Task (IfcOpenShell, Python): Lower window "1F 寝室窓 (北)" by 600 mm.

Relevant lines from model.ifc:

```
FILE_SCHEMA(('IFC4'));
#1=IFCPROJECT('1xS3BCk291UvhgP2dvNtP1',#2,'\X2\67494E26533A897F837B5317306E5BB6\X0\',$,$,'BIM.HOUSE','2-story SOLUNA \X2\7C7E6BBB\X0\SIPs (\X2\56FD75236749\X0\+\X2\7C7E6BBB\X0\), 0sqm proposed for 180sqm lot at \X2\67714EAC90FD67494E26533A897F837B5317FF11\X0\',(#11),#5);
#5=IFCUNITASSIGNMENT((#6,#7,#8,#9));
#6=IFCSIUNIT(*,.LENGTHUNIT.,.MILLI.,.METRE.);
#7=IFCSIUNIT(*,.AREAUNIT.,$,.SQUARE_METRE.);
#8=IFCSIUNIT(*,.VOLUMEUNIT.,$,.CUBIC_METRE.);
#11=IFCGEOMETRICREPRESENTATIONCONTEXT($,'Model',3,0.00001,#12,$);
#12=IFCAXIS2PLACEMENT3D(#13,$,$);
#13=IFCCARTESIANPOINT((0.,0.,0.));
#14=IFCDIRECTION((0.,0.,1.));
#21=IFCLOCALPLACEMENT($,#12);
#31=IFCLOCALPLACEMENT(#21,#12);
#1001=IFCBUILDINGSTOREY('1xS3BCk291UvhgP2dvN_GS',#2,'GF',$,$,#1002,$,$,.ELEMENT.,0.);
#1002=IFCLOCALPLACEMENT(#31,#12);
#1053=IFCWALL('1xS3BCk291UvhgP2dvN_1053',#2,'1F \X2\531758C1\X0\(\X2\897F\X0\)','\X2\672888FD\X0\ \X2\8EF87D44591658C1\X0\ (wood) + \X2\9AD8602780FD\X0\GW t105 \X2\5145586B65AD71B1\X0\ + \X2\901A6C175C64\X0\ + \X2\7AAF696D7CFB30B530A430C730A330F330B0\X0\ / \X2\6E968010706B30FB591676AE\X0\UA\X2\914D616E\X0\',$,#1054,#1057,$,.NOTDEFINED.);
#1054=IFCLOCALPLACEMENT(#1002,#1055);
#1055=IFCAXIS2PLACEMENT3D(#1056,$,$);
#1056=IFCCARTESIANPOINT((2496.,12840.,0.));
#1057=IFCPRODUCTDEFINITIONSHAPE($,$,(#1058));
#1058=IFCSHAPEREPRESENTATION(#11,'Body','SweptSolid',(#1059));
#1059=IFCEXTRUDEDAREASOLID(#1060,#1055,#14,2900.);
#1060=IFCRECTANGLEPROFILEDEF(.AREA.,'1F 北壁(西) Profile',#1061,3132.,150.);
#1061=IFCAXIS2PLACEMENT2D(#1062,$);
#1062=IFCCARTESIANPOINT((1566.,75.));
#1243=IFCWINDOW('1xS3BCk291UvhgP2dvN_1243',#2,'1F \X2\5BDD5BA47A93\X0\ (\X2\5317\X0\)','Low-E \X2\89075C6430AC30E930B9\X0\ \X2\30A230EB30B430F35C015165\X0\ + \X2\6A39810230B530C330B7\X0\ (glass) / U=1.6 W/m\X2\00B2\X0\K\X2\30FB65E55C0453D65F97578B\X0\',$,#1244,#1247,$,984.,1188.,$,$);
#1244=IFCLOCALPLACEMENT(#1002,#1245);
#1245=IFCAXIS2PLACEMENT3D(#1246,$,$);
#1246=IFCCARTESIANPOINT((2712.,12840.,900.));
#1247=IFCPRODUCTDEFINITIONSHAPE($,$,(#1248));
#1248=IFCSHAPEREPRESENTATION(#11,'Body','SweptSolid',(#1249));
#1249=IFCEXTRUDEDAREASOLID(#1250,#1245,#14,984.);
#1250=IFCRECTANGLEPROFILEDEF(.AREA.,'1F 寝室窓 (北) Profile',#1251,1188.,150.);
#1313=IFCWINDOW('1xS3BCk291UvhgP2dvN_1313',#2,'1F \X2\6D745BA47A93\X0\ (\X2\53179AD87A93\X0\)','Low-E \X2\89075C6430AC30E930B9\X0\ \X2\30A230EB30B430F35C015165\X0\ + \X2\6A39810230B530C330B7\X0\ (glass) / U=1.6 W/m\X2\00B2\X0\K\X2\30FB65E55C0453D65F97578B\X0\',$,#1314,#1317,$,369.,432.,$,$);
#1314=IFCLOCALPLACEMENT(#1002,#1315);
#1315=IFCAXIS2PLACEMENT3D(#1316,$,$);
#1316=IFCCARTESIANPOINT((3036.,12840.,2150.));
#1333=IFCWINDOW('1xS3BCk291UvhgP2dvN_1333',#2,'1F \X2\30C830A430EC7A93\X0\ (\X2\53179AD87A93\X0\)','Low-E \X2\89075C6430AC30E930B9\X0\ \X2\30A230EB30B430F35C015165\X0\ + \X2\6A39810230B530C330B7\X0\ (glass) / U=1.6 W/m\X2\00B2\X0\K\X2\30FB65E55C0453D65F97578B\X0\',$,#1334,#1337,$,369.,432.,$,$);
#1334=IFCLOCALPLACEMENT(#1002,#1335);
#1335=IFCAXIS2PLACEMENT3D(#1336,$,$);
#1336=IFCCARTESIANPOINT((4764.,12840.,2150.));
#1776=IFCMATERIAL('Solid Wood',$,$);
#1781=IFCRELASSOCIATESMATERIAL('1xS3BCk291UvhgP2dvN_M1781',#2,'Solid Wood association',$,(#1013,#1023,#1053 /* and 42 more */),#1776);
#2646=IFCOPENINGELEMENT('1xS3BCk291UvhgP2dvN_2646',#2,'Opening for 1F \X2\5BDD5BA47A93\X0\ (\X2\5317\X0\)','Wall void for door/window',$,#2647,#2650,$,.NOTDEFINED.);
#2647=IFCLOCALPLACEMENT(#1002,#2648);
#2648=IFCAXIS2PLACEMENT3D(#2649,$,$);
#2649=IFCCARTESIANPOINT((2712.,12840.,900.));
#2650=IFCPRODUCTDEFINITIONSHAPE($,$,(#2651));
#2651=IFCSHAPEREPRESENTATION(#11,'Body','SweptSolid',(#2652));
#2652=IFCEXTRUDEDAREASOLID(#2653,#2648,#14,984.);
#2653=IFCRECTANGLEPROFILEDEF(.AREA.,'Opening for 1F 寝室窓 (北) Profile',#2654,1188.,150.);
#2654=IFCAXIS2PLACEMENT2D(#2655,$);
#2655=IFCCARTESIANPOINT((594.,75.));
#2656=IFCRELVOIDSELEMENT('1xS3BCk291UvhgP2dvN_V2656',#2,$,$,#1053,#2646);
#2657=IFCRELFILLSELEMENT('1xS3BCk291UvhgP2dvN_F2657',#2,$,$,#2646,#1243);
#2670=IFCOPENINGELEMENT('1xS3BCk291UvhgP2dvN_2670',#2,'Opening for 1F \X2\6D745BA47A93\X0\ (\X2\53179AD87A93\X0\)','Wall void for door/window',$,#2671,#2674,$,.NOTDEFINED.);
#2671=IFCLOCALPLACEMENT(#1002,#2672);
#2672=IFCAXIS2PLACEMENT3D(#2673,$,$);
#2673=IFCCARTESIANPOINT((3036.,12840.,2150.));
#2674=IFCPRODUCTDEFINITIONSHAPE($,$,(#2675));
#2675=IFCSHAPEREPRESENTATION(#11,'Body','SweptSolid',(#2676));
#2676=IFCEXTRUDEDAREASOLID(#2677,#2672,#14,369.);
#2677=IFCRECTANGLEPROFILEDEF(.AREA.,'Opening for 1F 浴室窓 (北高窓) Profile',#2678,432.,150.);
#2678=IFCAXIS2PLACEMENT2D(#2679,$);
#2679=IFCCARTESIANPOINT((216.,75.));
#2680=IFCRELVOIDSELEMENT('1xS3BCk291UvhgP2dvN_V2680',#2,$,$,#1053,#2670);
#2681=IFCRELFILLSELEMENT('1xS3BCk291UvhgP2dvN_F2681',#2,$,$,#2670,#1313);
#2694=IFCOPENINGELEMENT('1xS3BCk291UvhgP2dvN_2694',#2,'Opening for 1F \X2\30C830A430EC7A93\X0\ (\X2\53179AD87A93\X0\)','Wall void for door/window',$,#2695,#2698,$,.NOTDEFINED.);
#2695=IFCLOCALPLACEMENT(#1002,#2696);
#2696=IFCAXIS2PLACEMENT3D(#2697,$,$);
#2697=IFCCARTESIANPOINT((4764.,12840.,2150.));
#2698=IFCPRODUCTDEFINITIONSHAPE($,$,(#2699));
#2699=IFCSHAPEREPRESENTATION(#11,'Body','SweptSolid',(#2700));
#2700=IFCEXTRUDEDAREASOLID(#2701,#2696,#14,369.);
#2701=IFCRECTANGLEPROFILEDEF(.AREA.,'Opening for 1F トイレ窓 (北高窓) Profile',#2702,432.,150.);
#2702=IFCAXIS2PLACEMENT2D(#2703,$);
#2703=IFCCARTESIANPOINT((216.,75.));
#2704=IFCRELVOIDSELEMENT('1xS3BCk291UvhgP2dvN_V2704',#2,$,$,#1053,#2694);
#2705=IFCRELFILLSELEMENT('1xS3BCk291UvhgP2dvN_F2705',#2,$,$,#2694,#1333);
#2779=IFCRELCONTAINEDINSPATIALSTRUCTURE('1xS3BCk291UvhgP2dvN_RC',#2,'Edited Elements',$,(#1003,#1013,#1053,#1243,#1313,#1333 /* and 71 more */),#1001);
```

```python
import numpy as np
import ifcopenshell
import ifcopenshell.api.geometry
import ifcopenshell.util.placement
import ifcopenshell.util.unit

model = ifcopenshell.open("model.ifc")
unit_scale = ifcopenshell.util.unit.calculate_unit_scale(model)

window = model.by_id(1243)
opening = window.FillsVoids[0].RelatingOpeningElement
dz = -0.6 / unit_scale

shift = np.array([0.0, 0.0, dz])
# The window is not placed relative to its opening, so move both.
for product in (opening, window):
    matrix = ifcopenshell.util.placement.get_local_placement(product.ObjectPlacement)
    matrix[:3, 3] += shift
    ifcopenshell.api.geometry.edit_object_placement(model, product=product, matrix=matrix, is_si=False)

print(f"moved by {dz * unit_scale:+.3f} m")

model.write("model_v2.ifc")
```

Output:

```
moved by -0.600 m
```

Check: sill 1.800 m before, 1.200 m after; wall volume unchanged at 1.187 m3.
